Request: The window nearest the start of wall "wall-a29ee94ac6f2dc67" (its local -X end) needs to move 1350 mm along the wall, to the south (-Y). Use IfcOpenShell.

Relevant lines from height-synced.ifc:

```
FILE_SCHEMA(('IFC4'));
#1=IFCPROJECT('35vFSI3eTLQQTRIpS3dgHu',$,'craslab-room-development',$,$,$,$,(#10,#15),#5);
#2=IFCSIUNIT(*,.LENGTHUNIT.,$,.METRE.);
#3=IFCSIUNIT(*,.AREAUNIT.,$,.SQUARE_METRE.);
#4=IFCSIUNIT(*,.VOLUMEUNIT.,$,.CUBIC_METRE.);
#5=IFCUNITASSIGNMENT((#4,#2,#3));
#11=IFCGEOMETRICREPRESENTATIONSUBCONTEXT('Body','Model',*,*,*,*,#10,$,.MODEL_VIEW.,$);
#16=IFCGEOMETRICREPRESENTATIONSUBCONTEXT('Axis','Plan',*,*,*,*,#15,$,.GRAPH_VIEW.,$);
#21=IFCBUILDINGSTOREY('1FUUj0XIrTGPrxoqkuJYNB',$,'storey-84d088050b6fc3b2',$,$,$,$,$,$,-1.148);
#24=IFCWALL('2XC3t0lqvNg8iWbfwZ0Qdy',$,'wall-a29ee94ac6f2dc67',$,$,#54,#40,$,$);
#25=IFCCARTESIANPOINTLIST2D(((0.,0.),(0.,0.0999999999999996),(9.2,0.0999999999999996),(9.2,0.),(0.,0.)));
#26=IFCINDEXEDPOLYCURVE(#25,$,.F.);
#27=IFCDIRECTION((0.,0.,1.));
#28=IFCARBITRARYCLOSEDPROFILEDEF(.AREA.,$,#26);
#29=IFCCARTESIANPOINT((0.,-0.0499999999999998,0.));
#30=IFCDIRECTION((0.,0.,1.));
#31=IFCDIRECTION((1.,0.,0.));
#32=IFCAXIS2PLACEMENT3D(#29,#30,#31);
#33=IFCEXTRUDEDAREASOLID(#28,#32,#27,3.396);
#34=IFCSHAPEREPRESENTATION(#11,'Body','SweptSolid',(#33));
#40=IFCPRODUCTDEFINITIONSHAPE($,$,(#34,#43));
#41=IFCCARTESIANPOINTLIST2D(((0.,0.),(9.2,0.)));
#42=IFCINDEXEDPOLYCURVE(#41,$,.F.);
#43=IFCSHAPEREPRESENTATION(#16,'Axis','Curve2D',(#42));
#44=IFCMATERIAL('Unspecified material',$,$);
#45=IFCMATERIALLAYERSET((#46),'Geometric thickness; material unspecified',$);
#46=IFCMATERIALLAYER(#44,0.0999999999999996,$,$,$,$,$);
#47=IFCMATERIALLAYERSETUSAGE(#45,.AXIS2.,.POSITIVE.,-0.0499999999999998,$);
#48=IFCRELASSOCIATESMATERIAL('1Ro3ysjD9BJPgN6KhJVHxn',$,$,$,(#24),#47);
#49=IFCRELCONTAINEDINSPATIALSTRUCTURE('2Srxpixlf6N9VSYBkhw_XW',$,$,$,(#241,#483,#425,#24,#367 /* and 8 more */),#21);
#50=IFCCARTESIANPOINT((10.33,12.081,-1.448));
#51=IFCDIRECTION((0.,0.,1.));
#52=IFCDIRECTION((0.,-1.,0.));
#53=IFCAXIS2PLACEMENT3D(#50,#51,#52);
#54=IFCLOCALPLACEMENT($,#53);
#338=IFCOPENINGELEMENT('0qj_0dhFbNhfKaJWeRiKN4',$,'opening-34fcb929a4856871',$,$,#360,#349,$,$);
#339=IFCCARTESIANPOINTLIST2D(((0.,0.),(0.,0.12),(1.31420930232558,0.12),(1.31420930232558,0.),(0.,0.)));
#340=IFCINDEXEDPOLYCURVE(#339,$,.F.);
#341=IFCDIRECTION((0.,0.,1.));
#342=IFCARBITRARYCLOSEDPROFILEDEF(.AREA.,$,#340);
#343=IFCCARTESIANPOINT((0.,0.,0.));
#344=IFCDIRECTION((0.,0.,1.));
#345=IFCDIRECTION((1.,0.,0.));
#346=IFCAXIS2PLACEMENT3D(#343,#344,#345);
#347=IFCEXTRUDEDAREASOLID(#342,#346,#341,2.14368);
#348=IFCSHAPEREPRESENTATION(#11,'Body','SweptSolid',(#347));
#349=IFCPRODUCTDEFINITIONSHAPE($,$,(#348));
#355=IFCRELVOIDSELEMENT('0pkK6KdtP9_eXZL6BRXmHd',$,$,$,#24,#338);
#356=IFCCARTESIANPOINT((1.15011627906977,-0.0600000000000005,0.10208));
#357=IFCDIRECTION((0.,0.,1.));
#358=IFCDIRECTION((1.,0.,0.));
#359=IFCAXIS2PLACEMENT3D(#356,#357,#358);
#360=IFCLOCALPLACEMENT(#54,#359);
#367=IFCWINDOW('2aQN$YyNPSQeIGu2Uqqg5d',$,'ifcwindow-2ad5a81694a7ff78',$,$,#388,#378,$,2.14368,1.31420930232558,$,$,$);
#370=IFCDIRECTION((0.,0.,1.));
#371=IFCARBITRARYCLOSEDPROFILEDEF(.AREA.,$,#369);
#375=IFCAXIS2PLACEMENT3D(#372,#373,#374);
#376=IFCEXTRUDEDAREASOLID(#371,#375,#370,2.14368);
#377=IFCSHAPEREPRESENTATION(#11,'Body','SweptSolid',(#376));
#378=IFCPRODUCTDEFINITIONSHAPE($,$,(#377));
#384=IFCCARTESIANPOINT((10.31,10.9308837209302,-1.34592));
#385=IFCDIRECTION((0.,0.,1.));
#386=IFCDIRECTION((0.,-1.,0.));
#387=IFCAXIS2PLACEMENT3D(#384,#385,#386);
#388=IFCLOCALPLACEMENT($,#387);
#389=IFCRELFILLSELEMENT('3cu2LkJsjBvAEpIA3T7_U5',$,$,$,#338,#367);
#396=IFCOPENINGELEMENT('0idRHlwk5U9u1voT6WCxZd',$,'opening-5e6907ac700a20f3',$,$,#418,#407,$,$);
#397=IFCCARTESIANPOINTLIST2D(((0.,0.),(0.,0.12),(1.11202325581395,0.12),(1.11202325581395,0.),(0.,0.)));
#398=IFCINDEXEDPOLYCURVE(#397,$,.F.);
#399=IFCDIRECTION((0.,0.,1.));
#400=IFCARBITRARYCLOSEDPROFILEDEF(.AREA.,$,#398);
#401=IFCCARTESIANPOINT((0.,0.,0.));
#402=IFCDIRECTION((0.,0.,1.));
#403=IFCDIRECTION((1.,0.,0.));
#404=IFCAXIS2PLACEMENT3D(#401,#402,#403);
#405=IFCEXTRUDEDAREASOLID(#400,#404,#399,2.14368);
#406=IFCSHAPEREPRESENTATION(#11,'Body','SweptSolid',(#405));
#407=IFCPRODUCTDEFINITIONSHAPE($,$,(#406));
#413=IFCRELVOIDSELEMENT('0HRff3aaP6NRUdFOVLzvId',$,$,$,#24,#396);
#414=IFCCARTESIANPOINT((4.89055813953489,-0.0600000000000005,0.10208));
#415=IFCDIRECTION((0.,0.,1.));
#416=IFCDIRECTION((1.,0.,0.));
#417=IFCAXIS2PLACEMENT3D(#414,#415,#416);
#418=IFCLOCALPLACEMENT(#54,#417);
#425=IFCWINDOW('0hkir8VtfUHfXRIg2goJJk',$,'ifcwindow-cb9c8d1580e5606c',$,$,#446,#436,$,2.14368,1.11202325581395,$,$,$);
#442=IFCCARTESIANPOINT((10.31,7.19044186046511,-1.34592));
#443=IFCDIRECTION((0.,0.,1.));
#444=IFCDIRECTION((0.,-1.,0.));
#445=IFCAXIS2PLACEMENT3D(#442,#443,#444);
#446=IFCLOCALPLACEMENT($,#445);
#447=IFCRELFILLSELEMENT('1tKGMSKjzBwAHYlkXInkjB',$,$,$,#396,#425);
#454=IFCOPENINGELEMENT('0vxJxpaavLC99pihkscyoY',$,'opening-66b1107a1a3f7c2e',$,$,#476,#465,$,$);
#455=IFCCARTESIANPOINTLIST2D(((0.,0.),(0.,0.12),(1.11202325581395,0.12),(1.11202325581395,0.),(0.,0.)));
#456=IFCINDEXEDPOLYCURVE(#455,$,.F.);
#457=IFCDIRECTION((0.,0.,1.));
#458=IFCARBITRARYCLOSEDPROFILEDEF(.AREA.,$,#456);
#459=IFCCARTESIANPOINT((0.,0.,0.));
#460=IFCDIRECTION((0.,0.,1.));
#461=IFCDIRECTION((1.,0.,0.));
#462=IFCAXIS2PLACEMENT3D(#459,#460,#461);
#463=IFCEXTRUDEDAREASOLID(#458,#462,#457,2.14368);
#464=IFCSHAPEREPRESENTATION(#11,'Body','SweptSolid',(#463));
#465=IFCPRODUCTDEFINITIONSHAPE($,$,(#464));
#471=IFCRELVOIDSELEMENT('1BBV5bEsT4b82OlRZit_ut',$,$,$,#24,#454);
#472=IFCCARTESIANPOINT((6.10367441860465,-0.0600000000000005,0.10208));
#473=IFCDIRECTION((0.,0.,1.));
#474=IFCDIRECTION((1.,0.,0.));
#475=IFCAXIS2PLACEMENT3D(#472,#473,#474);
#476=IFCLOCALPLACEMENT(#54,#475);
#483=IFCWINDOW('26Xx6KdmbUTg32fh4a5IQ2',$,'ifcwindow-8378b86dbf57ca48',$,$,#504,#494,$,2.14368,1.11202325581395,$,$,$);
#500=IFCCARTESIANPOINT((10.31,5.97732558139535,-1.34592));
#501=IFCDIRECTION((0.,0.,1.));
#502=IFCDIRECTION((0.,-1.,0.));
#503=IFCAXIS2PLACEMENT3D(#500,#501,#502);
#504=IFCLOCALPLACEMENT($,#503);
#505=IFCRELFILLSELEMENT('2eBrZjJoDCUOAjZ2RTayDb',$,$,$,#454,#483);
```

```python
import ifcopenshell
import ifcopenshell.api.geometry
import ifcopenshell.util.placement

model = ifcopenshell.open("height-synced.ifc")

window = model.by_guid("2aQN$YyNPSQeIGu2Uqqg5d")
opening = window.FillsVoids[0].RelatingOpeningElement
wall = opening.VoidsElements[0].RelatingBuildingElement

wall_matrix = ifcopenshell.util.placement.get_local_placement(wall.ObjectPlacement)
shift = wall_matrix[:3, 0] * 1.35
before = ifcopenshell.util.placement.get_local_placement(window.ObjectPlacement)[:3, 3].copy()

# The window is not placed relative to its opening, so move both.
for product in (opening, window):
    matrix = ifcopenshell.util.placement.get_local_placement(product.ObjectPlacement)
    matrix[:3, 3] += shift
    ifcopenshell.api.geometry.edit_object_placement(model, product=product, matrix=matrix, is_si=False)

after = ifcopenshell.util.placement.get_local_placement(window.ObjectPlacement)[:3, 3]
print("window moved by", (after - before).round(3) + 0.0)

model.write("height-synced-out.ifc")
```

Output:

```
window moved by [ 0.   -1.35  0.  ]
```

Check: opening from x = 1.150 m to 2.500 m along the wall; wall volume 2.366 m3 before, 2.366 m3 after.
